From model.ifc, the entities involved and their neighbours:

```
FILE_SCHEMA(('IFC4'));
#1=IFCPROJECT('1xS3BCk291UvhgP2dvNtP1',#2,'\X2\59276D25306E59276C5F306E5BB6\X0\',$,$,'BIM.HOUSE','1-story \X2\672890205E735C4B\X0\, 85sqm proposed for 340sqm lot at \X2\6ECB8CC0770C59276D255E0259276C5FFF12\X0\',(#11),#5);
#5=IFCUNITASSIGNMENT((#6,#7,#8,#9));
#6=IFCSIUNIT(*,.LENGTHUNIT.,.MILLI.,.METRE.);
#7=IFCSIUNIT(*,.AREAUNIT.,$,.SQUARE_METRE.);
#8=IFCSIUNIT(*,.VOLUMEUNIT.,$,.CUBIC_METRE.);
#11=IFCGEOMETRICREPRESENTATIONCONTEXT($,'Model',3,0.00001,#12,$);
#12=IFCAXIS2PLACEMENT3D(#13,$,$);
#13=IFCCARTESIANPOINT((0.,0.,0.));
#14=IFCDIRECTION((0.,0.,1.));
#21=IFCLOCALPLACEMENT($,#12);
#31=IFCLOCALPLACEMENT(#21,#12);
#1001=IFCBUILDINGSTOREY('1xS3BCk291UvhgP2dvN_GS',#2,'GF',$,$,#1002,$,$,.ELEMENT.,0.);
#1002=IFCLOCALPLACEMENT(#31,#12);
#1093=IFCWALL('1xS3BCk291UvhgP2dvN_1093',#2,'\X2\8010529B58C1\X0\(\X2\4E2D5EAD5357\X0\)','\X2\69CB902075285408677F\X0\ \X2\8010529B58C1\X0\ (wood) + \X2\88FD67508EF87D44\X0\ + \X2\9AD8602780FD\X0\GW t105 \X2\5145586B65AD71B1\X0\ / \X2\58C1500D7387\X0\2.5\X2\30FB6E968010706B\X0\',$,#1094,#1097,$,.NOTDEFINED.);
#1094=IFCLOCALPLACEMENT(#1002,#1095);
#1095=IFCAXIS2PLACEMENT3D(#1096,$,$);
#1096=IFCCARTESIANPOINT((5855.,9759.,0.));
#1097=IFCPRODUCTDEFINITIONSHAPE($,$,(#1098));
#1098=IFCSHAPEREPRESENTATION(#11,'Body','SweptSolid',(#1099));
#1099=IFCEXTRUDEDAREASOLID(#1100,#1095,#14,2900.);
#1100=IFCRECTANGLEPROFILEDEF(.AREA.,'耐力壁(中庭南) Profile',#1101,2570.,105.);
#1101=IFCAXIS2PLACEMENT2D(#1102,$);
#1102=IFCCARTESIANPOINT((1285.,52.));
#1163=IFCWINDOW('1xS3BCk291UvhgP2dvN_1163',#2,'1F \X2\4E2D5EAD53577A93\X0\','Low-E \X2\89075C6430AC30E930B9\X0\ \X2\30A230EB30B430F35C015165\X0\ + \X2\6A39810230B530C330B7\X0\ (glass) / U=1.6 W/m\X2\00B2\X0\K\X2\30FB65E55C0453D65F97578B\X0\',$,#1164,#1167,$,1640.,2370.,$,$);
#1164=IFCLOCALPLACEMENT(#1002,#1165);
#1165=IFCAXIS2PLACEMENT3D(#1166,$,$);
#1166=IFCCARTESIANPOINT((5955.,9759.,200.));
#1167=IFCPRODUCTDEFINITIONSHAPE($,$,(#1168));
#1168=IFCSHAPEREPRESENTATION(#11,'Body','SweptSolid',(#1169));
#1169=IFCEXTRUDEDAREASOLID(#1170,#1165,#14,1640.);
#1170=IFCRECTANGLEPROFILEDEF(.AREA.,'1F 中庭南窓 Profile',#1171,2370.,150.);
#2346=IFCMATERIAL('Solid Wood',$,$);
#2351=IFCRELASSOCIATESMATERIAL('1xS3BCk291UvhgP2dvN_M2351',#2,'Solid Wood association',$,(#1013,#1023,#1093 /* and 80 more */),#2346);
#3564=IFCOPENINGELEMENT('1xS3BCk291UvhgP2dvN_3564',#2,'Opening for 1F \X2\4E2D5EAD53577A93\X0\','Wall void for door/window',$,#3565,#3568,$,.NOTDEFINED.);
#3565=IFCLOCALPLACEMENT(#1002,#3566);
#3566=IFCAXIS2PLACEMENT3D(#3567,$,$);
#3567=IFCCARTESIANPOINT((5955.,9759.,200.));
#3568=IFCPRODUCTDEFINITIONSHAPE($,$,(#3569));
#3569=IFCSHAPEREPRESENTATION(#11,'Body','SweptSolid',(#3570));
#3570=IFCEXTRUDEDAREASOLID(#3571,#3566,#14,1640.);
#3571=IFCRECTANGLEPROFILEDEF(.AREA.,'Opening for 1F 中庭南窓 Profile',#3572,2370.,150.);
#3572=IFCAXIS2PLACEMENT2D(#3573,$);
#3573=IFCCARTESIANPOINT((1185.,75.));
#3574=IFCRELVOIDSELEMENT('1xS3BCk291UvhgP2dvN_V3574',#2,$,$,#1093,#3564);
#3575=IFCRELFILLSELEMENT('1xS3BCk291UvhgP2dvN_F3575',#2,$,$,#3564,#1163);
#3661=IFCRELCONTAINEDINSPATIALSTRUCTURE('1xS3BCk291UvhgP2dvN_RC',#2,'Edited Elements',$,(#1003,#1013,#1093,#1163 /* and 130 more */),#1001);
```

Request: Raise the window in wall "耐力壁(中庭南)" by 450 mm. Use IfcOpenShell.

```python
import numpy as np
import ifcopenshell
import ifcopenshell.api.geometry
import ifcopenshell.util.placement
import ifcopenshell.util.unit

model = ifcopenshell.open("model.ifc")
unit_scale = ifcopenshell.util.unit.calculate_unit_scale(model)

window = model.by_guid("1xS3BCk291UvhgP2dvN_1163")
opening = window.FillsVoids[0].RelatingOpeningElement
dz = 450.0

shift = np.array([0.0, 0.0, dz])
# The window is not placed relative to its opening, so move both.
for product in (opening, window):
    matrix = ifcopenshell.util.placement.get_local_placement(product.ObjectPlacement)
    matrix[:3, 3] += shift
    ifcopenshell.api.geometry.edit_object_placement(model, product=product, matrix=matrix, is_si=False)

print(f"moved by {dz * unit_scale:+.3f} m")

model.write("model_v2.ifc")
```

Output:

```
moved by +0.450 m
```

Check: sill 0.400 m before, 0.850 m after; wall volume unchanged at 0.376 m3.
